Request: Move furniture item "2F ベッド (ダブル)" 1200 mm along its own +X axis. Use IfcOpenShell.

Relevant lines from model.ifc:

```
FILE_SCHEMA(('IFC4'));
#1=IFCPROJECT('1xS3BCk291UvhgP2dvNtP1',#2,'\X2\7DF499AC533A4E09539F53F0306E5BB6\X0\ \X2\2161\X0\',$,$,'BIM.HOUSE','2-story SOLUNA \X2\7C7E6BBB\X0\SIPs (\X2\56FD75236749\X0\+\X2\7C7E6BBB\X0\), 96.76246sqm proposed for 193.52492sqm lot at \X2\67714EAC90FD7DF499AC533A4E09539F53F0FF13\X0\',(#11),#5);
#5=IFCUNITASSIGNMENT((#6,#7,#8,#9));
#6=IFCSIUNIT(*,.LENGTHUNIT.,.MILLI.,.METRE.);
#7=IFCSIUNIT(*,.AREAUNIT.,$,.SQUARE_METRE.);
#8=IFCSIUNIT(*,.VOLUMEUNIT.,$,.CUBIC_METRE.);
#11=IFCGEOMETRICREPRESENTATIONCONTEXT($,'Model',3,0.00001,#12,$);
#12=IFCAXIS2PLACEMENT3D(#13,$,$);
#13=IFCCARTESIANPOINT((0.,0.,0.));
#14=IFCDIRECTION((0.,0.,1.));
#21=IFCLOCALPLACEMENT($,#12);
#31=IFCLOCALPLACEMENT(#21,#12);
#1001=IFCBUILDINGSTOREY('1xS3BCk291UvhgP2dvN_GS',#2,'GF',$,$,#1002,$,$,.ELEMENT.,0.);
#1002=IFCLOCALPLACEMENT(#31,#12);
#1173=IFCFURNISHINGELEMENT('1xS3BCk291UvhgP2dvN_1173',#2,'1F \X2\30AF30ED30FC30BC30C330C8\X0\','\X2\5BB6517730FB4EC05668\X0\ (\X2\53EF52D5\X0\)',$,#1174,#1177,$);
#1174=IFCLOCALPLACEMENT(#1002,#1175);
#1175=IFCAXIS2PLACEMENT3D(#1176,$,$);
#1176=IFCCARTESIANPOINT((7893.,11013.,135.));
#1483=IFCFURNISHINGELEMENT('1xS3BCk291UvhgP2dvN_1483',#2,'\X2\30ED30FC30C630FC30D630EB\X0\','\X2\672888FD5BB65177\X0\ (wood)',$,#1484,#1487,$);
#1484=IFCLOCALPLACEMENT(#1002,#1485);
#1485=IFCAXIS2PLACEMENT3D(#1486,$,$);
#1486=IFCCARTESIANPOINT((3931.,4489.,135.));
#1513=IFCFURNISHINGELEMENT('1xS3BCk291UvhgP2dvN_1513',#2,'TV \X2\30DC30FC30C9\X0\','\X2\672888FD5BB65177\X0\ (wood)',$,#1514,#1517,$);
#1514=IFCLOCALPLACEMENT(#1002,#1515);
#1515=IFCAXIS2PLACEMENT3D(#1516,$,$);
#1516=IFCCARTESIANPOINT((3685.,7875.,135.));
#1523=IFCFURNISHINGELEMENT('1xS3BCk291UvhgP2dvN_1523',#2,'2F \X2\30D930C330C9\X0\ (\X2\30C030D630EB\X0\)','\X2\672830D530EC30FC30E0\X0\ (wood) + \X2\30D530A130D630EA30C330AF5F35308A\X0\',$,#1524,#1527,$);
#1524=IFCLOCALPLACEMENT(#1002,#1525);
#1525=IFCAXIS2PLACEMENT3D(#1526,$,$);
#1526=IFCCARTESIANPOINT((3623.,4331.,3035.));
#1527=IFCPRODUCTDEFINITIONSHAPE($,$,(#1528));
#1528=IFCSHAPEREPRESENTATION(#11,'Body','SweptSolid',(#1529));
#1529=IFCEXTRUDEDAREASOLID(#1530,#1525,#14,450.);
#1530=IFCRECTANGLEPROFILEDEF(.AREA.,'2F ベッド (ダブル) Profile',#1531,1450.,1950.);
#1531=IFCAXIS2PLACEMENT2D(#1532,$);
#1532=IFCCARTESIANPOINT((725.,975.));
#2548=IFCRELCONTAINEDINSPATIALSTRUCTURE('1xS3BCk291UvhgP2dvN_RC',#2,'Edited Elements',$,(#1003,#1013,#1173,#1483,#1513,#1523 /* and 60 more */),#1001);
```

```python
import ifcopenshell
import ifcopenshell.api.geometry
import ifcopenshell.util.placement

model = ifcopenshell.open("model.ifc")

item = model.by_guid("1xS3BCk291UvhgP2dvN_1523")
matrix = ifcopenshell.util.placement.get_local_placement(item.ObjectPlacement)
matrix[:3, 3] += matrix[:3, 0] * 1200.0
ifcopenshell.api.geometry.edit_object_placement(model, product=item, matrix=matrix, is_si=False)

print(ifcopenshell.util.placement.get_local_placement(item.ObjectPlacement).round(3) + 0.0)

model.write("model_updated.ifc")
```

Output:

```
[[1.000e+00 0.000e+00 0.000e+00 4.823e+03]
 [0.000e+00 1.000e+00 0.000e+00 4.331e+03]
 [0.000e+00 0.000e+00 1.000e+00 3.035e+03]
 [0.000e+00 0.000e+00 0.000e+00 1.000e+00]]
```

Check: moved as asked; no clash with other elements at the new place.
